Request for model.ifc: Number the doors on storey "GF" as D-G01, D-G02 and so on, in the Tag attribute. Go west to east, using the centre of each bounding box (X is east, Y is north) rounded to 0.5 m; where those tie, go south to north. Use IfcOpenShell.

First a look at what the model holds.

```python
import ifcopenshell
import ifcopenshell.util.element
import ifcopenshell.util.placement

model = ifcopenshell.open("model.ifc")
print(model.schema)
storey = next(s for s in model.by_type("IfcBuildingStorey") if s.Name == "GF")
doors = [e for e in ifcopenshell.util.element.get_decomposition(storey) if e.is_a("IfcDoor")]
for e in sorted(doors, key=lambda e: e.id()):
    origin = ifcopenshell.util.placement.get_local_placement(e.ObjectPlacement)[:3, 3]
    print(e.id(), e.Tag, e.Name, origin.round(2) + 0.0, sep=" | ")
```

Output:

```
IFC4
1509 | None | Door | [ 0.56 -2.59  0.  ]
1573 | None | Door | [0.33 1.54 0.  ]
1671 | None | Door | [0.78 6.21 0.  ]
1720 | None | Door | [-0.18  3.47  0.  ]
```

```python
import ifcopenshell
import ifcopenshell.geom
import ifcopenshell.util.element
import ifcopenshell.util.shape

model = ifcopenshell.open("model.ifc")
settings = ifcopenshell.geom.settings()
settings.set("use-world-coords", True)


def centre(element):
    shape = ifcopenshell.geom.create_shape(settings, element)
    return ifcopenshell.util.shape.get_bbox_centroid(shape.geometry)


storey = next(s for s in model.by_type("IfcBuildingStorey") if s.Name == "GF")
doors = [e for e in ifcopenshell.util.element.get_decomposition(storey) if e.is_a("IfcDoor")]

# Insertion points can sit at a corner or the storey origin, so sort by the geometry (in metres).
centres = {e: centre(e) for e in doors}
doors.sort(key=lambda e: (round(centres[e][0] / 0.5), centres[e][1]))

for i, e in enumerate(doors, start=1):
    number = f"D-G{i:02d}"
    e.Tag = number
    print(e.id(), number)

model.write("model_rev.ifc")
```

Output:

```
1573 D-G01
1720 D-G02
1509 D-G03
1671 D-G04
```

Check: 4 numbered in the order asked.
